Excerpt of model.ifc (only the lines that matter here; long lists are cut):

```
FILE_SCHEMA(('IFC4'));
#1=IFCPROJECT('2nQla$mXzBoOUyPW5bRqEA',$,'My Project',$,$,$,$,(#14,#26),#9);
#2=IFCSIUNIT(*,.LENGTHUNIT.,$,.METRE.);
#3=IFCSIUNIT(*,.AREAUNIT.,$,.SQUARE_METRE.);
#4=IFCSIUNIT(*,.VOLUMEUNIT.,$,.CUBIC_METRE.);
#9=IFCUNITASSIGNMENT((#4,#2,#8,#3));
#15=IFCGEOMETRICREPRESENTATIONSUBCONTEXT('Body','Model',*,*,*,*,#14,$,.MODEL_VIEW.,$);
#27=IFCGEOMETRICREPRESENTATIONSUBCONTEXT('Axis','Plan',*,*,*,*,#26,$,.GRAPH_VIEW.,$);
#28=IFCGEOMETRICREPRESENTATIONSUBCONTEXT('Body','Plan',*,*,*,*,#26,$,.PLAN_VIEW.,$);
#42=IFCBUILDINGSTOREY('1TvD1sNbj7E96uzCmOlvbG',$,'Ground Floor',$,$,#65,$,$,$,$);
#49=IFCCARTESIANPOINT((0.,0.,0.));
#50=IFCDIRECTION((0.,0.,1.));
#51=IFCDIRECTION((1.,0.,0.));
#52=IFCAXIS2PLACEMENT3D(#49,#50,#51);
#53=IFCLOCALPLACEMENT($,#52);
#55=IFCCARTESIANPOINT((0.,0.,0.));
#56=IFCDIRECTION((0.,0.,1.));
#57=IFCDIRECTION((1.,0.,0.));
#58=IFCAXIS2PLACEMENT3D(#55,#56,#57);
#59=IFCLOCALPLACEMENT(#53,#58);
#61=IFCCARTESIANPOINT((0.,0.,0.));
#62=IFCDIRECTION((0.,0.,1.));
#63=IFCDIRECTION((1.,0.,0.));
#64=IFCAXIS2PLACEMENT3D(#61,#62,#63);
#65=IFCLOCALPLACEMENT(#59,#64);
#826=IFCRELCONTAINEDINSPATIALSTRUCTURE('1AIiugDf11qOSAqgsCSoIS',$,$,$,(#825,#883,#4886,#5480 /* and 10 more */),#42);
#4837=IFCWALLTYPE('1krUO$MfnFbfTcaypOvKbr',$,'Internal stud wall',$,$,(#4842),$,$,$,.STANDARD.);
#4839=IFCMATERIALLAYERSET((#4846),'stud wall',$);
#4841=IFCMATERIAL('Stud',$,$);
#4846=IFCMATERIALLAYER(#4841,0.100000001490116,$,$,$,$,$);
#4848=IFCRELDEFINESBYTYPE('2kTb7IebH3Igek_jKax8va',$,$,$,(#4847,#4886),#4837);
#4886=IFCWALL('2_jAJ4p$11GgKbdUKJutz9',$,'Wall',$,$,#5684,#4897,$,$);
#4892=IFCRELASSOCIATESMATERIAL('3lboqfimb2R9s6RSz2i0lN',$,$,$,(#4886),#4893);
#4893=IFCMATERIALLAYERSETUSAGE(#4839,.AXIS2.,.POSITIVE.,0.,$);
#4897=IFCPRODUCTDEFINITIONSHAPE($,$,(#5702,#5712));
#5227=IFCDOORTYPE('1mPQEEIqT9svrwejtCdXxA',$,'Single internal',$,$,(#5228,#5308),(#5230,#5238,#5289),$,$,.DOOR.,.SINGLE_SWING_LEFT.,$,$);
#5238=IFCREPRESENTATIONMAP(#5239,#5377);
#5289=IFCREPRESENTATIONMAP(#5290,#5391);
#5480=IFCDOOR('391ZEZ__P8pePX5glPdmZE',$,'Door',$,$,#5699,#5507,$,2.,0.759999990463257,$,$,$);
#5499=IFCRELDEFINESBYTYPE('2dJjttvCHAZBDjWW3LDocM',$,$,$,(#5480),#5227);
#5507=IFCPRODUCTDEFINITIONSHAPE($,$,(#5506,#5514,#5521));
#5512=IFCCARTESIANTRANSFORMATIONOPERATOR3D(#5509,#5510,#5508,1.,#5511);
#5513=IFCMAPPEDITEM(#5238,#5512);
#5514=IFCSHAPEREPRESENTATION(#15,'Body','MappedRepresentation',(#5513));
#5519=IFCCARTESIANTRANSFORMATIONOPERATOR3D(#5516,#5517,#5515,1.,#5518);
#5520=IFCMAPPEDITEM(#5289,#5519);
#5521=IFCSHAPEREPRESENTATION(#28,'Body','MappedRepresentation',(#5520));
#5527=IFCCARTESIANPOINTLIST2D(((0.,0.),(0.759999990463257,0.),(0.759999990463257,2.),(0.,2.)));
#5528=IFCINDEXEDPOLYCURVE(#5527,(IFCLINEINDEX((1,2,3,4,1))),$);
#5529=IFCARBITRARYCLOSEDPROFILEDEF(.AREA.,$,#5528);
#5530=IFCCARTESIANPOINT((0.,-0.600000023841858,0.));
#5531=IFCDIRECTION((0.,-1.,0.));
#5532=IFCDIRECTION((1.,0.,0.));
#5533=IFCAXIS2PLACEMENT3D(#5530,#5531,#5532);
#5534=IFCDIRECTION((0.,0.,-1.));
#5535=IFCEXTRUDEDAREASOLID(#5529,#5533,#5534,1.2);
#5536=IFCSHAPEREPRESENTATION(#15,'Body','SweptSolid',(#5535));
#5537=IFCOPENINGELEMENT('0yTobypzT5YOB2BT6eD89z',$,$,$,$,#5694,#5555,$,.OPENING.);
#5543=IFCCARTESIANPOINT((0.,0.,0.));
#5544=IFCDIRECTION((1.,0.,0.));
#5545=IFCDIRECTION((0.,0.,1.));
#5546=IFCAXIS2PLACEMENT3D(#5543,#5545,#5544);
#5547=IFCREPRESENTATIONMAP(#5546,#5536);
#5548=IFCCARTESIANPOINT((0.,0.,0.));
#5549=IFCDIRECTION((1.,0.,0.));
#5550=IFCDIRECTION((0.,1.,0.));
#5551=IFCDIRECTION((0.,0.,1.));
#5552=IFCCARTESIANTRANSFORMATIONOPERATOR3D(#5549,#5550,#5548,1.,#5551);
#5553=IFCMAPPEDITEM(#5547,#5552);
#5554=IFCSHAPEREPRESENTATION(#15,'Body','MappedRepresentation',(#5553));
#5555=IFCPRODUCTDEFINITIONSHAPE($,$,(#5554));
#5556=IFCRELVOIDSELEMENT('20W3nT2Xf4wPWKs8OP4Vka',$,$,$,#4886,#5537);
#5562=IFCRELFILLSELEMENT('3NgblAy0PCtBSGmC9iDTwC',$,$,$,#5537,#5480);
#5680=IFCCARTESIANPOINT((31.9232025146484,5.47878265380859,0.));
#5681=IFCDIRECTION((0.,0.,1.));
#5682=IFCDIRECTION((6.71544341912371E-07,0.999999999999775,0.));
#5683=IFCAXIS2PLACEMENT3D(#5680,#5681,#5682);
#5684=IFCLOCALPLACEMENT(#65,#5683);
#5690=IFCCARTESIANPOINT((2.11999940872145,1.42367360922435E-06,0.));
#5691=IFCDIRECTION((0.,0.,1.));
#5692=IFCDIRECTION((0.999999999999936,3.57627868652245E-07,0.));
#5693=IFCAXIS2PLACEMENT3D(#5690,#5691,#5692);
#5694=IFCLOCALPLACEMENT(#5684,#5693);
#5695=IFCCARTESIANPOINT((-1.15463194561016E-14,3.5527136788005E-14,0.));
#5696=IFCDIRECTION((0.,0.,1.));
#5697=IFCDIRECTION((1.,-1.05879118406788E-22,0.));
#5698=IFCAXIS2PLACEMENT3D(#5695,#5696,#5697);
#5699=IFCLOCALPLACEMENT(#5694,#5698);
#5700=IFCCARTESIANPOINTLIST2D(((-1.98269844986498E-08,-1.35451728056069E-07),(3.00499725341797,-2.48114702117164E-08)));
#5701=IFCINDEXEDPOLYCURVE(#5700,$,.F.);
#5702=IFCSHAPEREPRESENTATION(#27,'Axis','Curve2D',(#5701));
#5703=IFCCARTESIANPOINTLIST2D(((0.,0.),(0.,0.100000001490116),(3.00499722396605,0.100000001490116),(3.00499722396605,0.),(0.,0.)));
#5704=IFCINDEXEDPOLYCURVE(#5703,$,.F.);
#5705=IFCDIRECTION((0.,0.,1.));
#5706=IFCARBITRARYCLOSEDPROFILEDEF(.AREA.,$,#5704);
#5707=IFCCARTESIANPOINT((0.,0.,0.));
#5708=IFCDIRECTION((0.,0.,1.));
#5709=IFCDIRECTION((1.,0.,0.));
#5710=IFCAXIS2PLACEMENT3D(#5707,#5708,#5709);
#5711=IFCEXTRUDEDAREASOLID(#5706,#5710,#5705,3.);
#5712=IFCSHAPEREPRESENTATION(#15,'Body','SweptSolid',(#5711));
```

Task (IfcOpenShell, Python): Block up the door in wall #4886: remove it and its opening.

```python
import ifcopenshell
import ifcopenshell.api.feature
import ifcopenshell.api.root
import ifcopenshell.geom
import ifcopenshell.util.shape

model = ifcopenshell.open("model.ifc")
settings = ifcopenshell.geom.settings()


def volume(element):
    """Net volume in cubic metres, openings subtracted."""
    shape = ifcopenshell.geom.create_shape(settings, element)
    return ifcopenshell.util.shape.get_volume(shape.geometry)


door = model.by_id(5480)
opening = door.FillsVoids[0].RelatingOpeningElement
wall = opening.VoidsElements[0].RelatingBuildingElement
before = volume(wall)

ifcopenshell.api.root.remove_product(model, product=door)
ifcopenshell.api.feature.remove_feature(model, feature=opening)

after = volume(wall)

print(f"wall volume {before:.3f} -> {after:.3f} m3")

model.write("model-out.ifc")
```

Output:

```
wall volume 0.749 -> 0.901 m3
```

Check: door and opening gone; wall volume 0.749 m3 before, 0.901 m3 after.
